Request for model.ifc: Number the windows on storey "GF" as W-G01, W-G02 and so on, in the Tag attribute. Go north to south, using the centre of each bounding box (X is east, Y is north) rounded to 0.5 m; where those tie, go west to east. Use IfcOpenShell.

First a look at what the model holds.

```python
import ifcopenshell
import ifcopenshell.util.element
import ifcopenshell.util.placement

model = ifcopenshell.open("model.ifc")
print(model.schema)
storey = next(s for s in model.by_type("IfcBuildingStorey") if s.Name == "GF")
windows = [e for e in ifcopenshell.util.element.get_decomposition(storey) if e.is_a("IfcWindow")]
for e in sorted(windows, key=lambda e: e.id()):
    origin = ifcopenshell.util.placement.get_local_placement(e.ObjectPlacement)[:3, 3]
    print(e.id(), e.Tag, e.Name, origin.round(2) + 0.0, sep=" | ")
```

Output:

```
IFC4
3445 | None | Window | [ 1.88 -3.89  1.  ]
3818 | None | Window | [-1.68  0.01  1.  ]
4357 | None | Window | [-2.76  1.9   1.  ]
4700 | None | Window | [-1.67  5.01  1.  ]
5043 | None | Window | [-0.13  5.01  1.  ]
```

```python
import ifcopenshell
import ifcopenshell.geom
import ifcopenshell.util.element
import ifcopenshell.util.shape

model = ifcopenshell.open("model.ifc")
settings = ifcopenshell.geom.settings()
settings.set("use-world-coords", True)


def centre(element):
    shape = ifcopenshell.geom.create_shape(settings, element)
    return ifcopenshell.util.shape.get_bbox_centroid(shape.geometry)


storey = next(s for s in model.by_type("IfcBuildingStorey") if s.Name == "GF")
windows = [e for e in ifcopenshell.util.element.get_decomposition(storey) if e.is_a("IfcWindow")]

# Insertion points can sit at a corner or the storey origin, so sort by the geometry (in metres).
centres = {e: centre(e) for e in windows}
windows.sort(key=lambda e: (-round(centres[e][1] / 0.5), centres[e][0]))

for i, e in enumerate(windows, start=1):
    number = f"W-G{i:02d}"
    e.Tag = number
    print(e.id(), number)

model.write("model_edited.ifc")
```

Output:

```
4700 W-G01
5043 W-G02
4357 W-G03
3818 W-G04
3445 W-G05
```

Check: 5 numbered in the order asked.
